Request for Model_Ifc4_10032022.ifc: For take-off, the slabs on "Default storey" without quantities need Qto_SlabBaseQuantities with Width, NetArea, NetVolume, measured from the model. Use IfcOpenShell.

First a look at what the model holds.

```python
import ifcopenshell
import ifcopenshell.util.element
import ifcopenshell.util.unit

model = ifcopenshell.open("Model_Ifc4_10032022.ifc")
print(model.schema)
for unit_type in ("LENGTHUNIT", "AREAUNIT", "VOLUMEUNIT"):
    print(unit_type, ifcopenshell.util.unit.calculate_unit_scale(model, unit_type))
storey = next(s for s in model.by_type("IfcBuildingStorey") if s.Name == "Default storey")
slabs = [e for e in ifcopenshell.util.element.get_decomposition(storey) if e.is_a("IfcSlab")]
for e in sorted(slabs, key=lambda e: e.id()):
    print(e.id(), e.is_a(), e.Name, list(ifcopenshell.util.element.get_psets(e, qtos_only=True)), sep=" | ")
```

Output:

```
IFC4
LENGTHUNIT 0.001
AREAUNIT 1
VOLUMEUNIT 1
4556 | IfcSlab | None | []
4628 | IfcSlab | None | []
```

```python
import ifcopenshell
import ifcopenshell.api.pset
import ifcopenshell.geom
import ifcopenshell.util.element
import ifcopenshell.util.shape
import ifcopenshell.util.unit

model = ifcopenshell.open("Model_Ifc4_10032022.ifc")
unit_scale = ifcopenshell.util.unit.calculate_unit_scale(model)
area_scale = ifcopenshell.util.unit.calculate_unit_scale(model, "AREAUNIT")
volume_scale = ifcopenshell.util.unit.calculate_unit_scale(model, "VOLUMEUNIT")
settings = ifcopenshell.geom.settings()

storey = next(s for s in model.by_type("IfcBuildingStorey") if s.Name == "Default storey")
slabs = [e for e in ifcopenshell.util.element.get_decomposition(storey) if e.is_a("IfcSlab")]

for e in sorted(slabs, key=lambda e: e.id()):
    if ifcopenshell.util.element.get_psets(e, qtos_only=True, should_inherit=False):
        continue
    # Geometry comes back in metres, in the element's own axes.
    shape = ifcopenshell.geom.create_shape(settings, e)
    values = {
        "Width": ifcopenshell.util.shape.get_z(shape.geometry) / unit_scale,
        "NetArea": ifcopenshell.util.shape.get_footprint_area(shape.geometry) / area_scale,
        "NetVolume": ifcopenshell.util.shape.get_volume(shape.geometry) / volume_scale,
    }
    qto = ifcopenshell.api.pset.add_qto(model, product=e, name="Qto_SlabBaseQuantities")
    ifcopenshell.api.pset.edit_qto(model, qto=qto, properties=values)
    print(e.id(), {k: round(v, 3) for k, v in values.items()})

model.write("Model_Ifc4_10032022_rev.ifc")
```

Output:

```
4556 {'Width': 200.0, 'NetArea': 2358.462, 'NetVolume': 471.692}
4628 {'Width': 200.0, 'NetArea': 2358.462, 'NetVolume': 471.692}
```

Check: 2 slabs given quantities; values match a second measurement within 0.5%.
